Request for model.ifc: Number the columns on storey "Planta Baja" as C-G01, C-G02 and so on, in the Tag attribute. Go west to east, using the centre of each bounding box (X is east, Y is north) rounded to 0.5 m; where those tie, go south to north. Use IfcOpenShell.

First a look at what the model holds.

```python
import ifcopenshell
import ifcopenshell.util.element
import ifcopenshell.util.placement

model = ifcopenshell.open("model.ifc")
print(model.schema)
storey = next(s for s in model.by_type("IfcBuildingStorey") if s.Name == "Planta Baja")
columns = [e for e in ifcopenshell.util.element.get_decomposition(storey) if e.is_a("IfcColumn")]
for e in sorted(columns, key=lambda e: e.id()):
    origin = ifcopenshell.util.placement.get_local_placement(e.ObjectPlacement)[:3, 3]
    print(e.id(), e.Tag, e.Name, origin.round(2) + 0.0, sep=" | ")
```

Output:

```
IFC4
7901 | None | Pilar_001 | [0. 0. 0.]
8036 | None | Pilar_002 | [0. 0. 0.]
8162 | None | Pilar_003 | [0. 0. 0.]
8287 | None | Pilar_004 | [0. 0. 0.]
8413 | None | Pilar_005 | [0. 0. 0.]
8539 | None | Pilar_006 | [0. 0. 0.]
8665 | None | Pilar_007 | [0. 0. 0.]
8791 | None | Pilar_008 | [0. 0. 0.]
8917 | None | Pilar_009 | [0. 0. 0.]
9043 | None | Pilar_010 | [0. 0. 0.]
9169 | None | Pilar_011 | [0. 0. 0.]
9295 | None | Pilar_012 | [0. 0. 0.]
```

```python
import ifcopenshell
import ifcopenshell.geom
import ifcopenshell.util.element
import ifcopenshell.util.shape

model = ifcopenshell.open("model.ifc")
settings = ifcopenshell.geom.settings()
settings.set("use-world-coords", True)


def centre(element):
    shape = ifcopenshell.geom.create_shape(settings, element)
    return ifcopenshell.util.shape.get_bbox_centroid(shape.geometry)


storey = next(s for s in model.by_type("IfcBuildingStorey") if s.Name == "Planta Baja")
columns = [e for e in ifcopenshell.util.element.get_decomposition(storey) if e.is_a("IfcColumn")]

# Insertion points can sit at a corner or the storey origin, so sort by the geometry (in metres).
centres = {e: centre(e) for e in columns}
columns.sort(key=lambda e: (round(centres[e][0] / 0.5), centres[e][1]))

for i, e in enumerate(columns, start=1):
    number = f"C-G{i:02d}"
    e.Tag = number
    print(e.id(), number)

model.write("model_edited.ifc")
```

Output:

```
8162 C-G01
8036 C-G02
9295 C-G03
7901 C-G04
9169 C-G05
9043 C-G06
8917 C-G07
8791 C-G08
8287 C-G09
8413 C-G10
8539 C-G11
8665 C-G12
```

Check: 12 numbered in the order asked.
